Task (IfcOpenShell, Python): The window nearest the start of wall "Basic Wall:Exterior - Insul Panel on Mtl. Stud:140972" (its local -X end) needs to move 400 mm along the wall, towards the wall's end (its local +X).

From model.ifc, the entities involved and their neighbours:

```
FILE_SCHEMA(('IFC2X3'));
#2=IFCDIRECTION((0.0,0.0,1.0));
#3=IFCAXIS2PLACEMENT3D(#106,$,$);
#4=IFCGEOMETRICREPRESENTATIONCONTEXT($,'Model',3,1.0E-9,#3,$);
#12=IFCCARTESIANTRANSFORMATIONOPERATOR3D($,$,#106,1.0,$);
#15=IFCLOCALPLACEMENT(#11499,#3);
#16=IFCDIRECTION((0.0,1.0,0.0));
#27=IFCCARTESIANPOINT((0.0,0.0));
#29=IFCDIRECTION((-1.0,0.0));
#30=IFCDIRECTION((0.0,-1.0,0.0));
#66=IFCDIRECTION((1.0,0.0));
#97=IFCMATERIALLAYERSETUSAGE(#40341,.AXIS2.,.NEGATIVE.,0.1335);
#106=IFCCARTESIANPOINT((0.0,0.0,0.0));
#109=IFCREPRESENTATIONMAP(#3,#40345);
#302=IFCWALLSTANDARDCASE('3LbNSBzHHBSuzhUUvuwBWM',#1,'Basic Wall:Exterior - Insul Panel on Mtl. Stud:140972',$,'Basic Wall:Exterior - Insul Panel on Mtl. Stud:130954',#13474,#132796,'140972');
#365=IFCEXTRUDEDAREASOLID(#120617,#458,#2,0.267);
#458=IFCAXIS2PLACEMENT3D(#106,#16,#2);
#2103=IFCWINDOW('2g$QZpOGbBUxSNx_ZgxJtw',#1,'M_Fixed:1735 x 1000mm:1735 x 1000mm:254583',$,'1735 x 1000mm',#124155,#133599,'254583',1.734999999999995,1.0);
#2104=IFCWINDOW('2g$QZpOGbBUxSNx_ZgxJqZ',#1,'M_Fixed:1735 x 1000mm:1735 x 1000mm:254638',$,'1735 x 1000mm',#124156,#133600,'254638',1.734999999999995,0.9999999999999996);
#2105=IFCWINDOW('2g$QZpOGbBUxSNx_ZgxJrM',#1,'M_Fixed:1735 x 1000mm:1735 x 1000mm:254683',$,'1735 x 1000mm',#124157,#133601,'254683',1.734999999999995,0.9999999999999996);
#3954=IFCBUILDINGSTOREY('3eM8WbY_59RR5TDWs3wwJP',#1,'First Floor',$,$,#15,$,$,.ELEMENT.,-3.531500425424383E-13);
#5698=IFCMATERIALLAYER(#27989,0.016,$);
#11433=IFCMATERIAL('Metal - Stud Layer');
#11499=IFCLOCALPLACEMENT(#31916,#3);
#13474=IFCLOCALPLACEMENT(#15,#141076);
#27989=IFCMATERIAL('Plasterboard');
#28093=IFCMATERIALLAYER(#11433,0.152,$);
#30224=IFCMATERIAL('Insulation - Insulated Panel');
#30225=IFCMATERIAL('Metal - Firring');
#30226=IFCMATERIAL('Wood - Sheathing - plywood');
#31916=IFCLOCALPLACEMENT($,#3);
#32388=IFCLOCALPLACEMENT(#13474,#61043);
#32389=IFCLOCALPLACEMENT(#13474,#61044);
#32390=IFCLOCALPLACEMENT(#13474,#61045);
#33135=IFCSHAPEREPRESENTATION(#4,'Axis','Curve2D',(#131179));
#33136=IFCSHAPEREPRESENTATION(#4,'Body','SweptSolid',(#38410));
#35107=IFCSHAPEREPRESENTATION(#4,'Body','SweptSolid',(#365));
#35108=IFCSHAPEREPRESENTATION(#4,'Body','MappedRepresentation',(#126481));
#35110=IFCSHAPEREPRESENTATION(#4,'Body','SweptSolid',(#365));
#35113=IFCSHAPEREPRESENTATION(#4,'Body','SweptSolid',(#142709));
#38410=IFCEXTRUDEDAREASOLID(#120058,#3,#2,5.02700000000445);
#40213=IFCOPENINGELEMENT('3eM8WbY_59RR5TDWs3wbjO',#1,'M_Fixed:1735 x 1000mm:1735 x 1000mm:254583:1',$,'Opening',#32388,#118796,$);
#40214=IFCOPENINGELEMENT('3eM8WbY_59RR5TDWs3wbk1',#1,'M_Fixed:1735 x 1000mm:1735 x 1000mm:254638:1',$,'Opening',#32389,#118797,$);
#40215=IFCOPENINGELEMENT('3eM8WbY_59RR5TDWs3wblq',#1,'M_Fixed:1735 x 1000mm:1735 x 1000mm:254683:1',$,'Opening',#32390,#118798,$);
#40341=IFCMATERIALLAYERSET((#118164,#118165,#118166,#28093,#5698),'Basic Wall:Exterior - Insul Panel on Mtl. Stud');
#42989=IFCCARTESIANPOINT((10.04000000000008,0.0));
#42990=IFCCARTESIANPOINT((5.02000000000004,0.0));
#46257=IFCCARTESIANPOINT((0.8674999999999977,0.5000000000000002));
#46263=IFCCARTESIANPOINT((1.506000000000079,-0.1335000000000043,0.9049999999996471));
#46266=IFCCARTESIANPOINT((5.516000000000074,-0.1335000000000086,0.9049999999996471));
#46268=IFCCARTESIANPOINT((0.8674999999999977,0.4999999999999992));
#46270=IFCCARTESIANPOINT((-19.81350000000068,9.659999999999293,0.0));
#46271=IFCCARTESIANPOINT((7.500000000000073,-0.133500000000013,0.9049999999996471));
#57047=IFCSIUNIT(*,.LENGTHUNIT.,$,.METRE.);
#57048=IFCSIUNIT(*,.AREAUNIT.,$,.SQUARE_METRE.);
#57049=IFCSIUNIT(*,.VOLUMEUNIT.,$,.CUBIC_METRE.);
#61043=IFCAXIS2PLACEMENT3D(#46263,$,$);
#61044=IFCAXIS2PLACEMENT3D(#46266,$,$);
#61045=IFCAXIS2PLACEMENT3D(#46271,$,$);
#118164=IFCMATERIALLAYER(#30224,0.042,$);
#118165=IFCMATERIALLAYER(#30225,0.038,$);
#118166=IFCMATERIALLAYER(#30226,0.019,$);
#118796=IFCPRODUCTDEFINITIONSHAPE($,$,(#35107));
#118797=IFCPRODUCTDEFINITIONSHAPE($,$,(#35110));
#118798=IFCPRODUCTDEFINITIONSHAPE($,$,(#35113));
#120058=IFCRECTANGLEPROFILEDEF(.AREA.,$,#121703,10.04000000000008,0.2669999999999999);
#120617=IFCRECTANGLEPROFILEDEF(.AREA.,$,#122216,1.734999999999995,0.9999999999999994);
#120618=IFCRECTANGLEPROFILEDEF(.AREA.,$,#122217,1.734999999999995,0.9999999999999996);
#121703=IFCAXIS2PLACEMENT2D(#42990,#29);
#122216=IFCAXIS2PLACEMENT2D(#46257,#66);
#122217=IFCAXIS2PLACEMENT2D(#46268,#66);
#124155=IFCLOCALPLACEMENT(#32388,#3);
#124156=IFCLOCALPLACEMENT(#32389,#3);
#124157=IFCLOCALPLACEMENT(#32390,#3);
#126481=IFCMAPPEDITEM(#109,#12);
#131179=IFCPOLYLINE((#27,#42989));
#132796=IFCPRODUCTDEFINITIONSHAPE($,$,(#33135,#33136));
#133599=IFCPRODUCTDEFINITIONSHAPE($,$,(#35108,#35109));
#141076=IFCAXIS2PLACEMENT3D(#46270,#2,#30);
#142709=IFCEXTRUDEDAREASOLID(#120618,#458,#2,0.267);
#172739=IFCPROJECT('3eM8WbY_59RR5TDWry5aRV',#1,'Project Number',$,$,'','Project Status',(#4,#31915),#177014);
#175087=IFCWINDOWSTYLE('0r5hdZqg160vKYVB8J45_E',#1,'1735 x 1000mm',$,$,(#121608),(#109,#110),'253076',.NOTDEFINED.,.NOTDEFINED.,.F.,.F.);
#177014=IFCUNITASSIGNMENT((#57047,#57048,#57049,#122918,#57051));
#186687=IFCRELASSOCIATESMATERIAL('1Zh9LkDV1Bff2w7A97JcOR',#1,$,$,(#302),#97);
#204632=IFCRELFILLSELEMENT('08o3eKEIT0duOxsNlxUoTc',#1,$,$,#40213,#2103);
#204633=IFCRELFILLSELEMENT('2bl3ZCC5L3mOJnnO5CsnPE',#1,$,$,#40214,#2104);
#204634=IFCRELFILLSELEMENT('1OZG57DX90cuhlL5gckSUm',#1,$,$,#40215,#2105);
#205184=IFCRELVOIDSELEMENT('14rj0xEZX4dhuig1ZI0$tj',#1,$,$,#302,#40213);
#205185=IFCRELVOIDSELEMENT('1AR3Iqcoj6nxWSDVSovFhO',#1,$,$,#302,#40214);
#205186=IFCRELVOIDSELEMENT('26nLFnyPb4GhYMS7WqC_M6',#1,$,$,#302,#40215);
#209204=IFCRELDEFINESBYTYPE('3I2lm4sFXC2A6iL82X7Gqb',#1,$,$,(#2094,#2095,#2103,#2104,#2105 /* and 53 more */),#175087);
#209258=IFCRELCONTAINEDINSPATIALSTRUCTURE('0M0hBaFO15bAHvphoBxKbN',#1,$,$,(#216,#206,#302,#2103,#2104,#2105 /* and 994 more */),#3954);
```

```python
import ifcopenshell
import ifcopenshell.api.geometry
import ifcopenshell.util.placement
import ifcopenshell.util.unit

model = ifcopenshell.open("model.ifc")
unit_scale = ifcopenshell.util.unit.calculate_unit_scale(model)

window = model.by_guid("2g$QZpOGbBUxSNx_ZgxJtw")
opening = window.FillsVoids[0].RelatingOpeningElement
wall = opening.VoidsElements[0].RelatingBuildingElement

wall_matrix = ifcopenshell.util.placement.get_local_placement(wall.ObjectPlacement)
shift = wall_matrix[:3, 0] * 0.4 / unit_scale
before = ifcopenshell.util.placement.get_local_placement(window.ObjectPlacement)[:3, 3].copy()

# The window is placed relative to its opening, so it follows when the opening moves.
matrix = ifcopenshell.util.placement.get_local_placement(opening.ObjectPlacement)
matrix[:3, 3] += shift
ifcopenshell.api.geometry.edit_object_placement(
    model, product=opening, matrix=matrix, is_si=False, should_transform_children=True
)

after = ifcopenshell.util.placement.get_local_placement(window.ObjectPlacement)[:3, 3]
print("window moved by", (after - before).round(3) + 0.0)

model.write("model_edited.ifc")
```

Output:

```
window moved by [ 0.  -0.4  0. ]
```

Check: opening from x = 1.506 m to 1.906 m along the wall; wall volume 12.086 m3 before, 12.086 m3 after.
